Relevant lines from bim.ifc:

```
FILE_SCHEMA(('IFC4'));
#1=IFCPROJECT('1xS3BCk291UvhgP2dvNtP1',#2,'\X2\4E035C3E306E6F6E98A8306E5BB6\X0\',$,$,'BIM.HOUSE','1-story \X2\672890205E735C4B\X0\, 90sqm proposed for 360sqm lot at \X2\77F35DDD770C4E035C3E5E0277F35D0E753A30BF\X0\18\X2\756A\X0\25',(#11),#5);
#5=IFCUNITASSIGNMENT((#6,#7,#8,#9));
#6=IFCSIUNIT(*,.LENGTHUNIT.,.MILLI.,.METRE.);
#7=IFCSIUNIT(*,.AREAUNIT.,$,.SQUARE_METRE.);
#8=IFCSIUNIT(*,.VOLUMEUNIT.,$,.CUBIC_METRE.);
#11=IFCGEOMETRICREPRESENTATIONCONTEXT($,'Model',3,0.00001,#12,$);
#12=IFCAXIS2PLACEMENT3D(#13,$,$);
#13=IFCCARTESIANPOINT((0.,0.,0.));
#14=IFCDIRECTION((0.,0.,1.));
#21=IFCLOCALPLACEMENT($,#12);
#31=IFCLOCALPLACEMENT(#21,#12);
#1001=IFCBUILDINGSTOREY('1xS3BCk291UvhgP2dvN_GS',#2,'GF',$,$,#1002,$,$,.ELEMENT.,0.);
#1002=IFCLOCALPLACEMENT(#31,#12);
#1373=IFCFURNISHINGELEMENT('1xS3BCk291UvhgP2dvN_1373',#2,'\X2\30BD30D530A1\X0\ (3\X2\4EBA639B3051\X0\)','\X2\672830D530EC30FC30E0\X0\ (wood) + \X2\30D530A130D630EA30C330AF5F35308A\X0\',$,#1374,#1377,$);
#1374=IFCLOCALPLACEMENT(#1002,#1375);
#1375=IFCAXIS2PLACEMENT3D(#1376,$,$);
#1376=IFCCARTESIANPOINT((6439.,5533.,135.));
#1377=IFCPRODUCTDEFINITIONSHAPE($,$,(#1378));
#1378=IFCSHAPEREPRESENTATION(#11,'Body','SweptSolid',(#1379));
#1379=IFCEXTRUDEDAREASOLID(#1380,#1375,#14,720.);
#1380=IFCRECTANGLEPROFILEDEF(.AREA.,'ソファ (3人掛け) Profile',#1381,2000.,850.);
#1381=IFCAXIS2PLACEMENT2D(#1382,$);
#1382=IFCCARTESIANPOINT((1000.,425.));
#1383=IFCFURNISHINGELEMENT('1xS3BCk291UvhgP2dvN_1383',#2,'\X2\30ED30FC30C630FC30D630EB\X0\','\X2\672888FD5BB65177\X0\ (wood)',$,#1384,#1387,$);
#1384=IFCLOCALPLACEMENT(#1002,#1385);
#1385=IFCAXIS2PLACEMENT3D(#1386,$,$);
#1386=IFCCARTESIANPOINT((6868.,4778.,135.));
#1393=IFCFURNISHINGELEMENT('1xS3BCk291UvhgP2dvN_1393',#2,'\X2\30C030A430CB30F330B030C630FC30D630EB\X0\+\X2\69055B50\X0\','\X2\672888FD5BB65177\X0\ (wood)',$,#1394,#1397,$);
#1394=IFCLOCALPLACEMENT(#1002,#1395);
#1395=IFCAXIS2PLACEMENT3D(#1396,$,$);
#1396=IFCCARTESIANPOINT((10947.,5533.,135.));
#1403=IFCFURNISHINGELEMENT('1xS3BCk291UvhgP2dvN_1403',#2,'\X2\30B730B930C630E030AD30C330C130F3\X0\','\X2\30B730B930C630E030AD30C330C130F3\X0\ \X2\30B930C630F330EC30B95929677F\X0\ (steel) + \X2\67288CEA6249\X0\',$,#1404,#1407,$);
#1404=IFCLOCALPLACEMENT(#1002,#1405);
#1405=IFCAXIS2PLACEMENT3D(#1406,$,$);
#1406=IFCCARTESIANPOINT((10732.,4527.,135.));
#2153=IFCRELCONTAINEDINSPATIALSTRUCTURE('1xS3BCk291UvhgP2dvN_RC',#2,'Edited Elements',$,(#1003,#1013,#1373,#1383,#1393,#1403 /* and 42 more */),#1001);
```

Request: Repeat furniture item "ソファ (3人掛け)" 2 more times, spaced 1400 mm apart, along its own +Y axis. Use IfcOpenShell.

```python
import ifcopenshell
import ifcopenshell.api.geometry
import ifcopenshell.api.root
import ifcopenshell.util.element
import ifcopenshell.util.placement

model = ifcopenshell.open("bim.ifc")


def reuse_history(source, copy):
    """copy_class also copies each property set's owner history, people and application; keep the originals."""
    for rel in copy.IsDefinedBy:
        if rel.is_a("IfcRelDefinesByProperties") and (history := rel.RelatingPropertyDefinition.OwnerHistory):
            rel.RelatingPropertyDefinition.OwnerHistory = source.OwnerHistory
            ifcopenshell.util.element.remove_deep2(model, history)


source = model.by_guid("1xS3BCk291UvhgP2dvN_1373")
base = ifcopenshell.util.placement.get_local_placement(source.ObjectPlacement)
step = base[:3, 1] * 1400.0

for i in range(1, 3):
    copy = ifcopenshell.api.root.copy_class(model, product=source)
    copy.Representation = ifcopenshell.util.element.copy_deep(
        model, source.Representation, exclude=["IfcGeometricRepresentationContext", "IfcRepresentationMap"]
    )
    reuse_history(source, copy)
    matrix = base.copy()
    matrix[:3, 3] += i * step
    print("added at", matrix[:3, 3].round(3) + 0.0)
    ifcopenshell.api.geometry.edit_object_placement(model, product=copy, matrix=matrix, is_si=False)

model.write("bim_rev.ifc")
```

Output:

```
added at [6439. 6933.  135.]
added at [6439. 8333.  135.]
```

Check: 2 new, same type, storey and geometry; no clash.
